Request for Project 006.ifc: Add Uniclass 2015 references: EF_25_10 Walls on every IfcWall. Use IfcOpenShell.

First a look at what the model holds.

```python
import ifcopenshell

model = ifcopenshell.open("Project 006.ifc")
print(model.schema)
print("classifications:", [c.Name for c in model.by_type("IfcClassification")])
for ifc_class in ("IfcDoor", "IfcRoof", "IfcStair", "IfcWall", "IfcWindow"):
    print(ifc_class, len(model.by_type(ifc_class)))
```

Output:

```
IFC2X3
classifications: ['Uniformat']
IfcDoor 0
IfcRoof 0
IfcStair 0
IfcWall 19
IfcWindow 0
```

```python
import ifcopenshell
import ifcopenshell.api.classification

model = ifcopenshell.open("Project 006.ifc")

# IFC2X3 requires Source and Edition and has no link from the project to the system.
system = model.create_entity("IfcClassification", Source="NBS", Edition="2015", Name="Uniclass 2015")

codes = {
    "IfcWall": ("EF_25_10", "Walls"),
}
for ifc_class, (code, name) in codes.items():
    products = model.by_type(ifc_class)
    ifcopenshell.api.classification.add_reference(
        model, products=products, classification=system, identification=code, name=name
    )
    print(code, len(products))

model.write("Project 006_edited.ifc")
```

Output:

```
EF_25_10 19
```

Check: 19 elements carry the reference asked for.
